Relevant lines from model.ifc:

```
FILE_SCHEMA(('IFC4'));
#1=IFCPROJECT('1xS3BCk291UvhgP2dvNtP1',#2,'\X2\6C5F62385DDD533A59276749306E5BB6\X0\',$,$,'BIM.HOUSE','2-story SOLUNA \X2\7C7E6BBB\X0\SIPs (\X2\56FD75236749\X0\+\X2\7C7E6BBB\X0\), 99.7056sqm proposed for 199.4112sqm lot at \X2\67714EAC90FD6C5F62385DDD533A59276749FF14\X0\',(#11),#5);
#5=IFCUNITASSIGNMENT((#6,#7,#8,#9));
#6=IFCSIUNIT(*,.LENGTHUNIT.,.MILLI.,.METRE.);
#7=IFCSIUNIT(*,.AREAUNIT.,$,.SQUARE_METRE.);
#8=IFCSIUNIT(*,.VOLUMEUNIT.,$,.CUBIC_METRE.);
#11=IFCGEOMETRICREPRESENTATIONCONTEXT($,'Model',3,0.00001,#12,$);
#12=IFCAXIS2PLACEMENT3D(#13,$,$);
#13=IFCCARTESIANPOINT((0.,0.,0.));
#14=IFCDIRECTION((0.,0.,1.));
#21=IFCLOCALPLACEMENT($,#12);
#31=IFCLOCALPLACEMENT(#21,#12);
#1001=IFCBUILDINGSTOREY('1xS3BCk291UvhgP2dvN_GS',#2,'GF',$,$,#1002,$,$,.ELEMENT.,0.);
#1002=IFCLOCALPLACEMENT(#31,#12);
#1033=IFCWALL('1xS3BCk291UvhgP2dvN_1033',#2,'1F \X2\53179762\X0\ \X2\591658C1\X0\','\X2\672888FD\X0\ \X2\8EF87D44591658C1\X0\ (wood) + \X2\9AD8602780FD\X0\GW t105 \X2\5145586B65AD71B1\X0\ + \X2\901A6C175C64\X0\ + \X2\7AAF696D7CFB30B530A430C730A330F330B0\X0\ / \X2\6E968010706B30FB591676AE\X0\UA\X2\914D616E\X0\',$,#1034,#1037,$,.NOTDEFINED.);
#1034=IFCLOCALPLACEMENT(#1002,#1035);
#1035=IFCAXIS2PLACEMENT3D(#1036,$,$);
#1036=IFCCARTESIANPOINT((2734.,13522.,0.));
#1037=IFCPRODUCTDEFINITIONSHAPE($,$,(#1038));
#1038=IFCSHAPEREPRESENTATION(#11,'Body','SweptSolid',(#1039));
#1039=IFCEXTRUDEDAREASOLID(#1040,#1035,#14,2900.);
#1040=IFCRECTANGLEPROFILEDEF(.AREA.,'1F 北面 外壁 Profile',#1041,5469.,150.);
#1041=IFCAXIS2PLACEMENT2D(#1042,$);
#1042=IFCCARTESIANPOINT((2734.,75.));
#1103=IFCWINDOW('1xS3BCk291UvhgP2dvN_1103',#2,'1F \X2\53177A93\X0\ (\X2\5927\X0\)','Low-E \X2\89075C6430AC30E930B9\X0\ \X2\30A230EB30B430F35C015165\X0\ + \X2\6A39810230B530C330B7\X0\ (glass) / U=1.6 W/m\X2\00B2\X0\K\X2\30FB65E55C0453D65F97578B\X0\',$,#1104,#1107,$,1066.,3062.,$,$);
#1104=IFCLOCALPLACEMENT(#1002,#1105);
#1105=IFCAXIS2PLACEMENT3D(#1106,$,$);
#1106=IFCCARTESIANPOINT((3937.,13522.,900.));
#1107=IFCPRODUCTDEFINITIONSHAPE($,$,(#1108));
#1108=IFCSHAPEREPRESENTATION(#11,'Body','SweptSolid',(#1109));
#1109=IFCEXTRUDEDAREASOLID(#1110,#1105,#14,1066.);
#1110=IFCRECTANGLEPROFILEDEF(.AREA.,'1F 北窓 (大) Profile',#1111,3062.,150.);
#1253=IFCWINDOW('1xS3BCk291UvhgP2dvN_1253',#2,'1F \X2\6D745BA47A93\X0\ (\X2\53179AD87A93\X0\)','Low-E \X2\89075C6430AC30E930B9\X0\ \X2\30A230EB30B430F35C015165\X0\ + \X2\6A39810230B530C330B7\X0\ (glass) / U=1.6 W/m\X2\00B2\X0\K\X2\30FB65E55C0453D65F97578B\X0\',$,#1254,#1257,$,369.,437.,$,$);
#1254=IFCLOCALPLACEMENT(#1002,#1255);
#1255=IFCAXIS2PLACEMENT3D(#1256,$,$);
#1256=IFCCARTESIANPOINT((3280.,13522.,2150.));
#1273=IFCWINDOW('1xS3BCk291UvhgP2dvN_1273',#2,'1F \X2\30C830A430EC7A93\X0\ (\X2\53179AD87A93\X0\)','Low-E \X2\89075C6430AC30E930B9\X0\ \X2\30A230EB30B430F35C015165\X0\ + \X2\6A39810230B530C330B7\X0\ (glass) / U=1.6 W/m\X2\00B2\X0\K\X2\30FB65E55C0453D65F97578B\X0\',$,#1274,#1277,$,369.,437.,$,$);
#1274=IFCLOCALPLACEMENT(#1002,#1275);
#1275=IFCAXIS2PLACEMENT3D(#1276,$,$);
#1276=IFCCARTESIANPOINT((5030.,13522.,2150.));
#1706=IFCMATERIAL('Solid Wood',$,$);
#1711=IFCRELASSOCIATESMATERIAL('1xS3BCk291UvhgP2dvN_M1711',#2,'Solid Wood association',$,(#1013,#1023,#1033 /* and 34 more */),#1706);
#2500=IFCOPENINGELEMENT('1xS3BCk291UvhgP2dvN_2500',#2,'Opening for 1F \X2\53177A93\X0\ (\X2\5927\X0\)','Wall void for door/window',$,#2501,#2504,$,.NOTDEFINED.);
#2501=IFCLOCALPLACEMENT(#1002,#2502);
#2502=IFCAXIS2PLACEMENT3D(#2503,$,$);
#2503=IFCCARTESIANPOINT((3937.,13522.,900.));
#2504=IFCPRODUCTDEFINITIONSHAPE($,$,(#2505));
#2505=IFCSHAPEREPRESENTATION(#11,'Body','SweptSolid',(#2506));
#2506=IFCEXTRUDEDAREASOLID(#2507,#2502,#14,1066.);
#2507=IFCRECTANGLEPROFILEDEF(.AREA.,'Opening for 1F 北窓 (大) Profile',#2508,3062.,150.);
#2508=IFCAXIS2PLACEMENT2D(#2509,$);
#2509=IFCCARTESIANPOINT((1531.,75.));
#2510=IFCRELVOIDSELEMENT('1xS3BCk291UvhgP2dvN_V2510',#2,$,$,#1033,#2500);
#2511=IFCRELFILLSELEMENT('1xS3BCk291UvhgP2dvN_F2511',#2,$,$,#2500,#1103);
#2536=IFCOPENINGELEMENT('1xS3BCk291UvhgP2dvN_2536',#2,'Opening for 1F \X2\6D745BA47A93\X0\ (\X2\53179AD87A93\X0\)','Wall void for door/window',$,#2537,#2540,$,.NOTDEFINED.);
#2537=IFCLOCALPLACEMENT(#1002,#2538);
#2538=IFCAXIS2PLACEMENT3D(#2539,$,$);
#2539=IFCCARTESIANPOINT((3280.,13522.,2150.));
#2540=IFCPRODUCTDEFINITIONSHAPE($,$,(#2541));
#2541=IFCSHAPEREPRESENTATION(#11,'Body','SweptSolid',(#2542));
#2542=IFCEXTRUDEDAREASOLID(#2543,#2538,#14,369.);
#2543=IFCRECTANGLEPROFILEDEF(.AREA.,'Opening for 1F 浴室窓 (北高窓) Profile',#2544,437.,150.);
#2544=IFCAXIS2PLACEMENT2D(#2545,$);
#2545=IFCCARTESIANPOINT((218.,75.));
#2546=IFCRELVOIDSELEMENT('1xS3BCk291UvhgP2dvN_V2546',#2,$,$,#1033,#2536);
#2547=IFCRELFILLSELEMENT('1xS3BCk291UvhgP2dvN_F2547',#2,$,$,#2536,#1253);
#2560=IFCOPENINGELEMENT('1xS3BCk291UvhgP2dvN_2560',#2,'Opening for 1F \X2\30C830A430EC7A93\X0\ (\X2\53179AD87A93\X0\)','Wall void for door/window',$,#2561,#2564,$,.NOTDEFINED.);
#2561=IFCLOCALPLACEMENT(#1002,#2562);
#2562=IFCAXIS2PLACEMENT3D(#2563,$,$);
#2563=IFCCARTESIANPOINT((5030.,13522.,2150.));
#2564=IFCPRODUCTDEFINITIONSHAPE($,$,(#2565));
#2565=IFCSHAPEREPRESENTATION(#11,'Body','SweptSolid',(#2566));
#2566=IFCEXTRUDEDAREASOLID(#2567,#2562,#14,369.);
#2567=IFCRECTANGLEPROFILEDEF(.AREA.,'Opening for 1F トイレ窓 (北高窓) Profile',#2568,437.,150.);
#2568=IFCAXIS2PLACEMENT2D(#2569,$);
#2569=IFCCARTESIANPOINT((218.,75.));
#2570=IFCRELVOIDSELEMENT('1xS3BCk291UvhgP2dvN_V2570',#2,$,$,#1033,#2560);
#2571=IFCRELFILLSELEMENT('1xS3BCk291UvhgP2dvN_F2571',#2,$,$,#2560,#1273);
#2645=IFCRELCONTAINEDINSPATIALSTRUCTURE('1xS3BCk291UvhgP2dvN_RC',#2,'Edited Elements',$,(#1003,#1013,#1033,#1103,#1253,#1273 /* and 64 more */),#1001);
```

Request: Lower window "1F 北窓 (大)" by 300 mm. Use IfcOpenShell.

```python
import numpy as np
import ifcopenshell
import ifcopenshell.api.geometry
import ifcopenshell.util.placement
import ifcopenshell.util.unit

model = ifcopenshell.open("model.ifc")
unit_scale = ifcopenshell.util.unit.calculate_unit_scale(model)

window = model.by_guid("1xS3BCk291UvhgP2dvN_1103")
opening = window.FillsVoids[0].RelatingOpeningElement
dz = -0.3 / unit_scale

shift = np.array([0.0, 0.0, dz])
# The window is not placed relative to its opening, so move both.
for product in (opening, window):
    matrix = ifcopenshell.util.placement.get_local_placement(product.ObjectPlacement)
    matrix[:3, 3] += shift
    ifcopenshell.api.geometry.edit_object_placement(model, product=product, matrix=matrix, is_si=False)

print(f"moved by {dz * unit_scale:+.3f} m")

model.write("model-out.ifc")
```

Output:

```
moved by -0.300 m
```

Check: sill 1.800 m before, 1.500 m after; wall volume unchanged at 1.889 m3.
